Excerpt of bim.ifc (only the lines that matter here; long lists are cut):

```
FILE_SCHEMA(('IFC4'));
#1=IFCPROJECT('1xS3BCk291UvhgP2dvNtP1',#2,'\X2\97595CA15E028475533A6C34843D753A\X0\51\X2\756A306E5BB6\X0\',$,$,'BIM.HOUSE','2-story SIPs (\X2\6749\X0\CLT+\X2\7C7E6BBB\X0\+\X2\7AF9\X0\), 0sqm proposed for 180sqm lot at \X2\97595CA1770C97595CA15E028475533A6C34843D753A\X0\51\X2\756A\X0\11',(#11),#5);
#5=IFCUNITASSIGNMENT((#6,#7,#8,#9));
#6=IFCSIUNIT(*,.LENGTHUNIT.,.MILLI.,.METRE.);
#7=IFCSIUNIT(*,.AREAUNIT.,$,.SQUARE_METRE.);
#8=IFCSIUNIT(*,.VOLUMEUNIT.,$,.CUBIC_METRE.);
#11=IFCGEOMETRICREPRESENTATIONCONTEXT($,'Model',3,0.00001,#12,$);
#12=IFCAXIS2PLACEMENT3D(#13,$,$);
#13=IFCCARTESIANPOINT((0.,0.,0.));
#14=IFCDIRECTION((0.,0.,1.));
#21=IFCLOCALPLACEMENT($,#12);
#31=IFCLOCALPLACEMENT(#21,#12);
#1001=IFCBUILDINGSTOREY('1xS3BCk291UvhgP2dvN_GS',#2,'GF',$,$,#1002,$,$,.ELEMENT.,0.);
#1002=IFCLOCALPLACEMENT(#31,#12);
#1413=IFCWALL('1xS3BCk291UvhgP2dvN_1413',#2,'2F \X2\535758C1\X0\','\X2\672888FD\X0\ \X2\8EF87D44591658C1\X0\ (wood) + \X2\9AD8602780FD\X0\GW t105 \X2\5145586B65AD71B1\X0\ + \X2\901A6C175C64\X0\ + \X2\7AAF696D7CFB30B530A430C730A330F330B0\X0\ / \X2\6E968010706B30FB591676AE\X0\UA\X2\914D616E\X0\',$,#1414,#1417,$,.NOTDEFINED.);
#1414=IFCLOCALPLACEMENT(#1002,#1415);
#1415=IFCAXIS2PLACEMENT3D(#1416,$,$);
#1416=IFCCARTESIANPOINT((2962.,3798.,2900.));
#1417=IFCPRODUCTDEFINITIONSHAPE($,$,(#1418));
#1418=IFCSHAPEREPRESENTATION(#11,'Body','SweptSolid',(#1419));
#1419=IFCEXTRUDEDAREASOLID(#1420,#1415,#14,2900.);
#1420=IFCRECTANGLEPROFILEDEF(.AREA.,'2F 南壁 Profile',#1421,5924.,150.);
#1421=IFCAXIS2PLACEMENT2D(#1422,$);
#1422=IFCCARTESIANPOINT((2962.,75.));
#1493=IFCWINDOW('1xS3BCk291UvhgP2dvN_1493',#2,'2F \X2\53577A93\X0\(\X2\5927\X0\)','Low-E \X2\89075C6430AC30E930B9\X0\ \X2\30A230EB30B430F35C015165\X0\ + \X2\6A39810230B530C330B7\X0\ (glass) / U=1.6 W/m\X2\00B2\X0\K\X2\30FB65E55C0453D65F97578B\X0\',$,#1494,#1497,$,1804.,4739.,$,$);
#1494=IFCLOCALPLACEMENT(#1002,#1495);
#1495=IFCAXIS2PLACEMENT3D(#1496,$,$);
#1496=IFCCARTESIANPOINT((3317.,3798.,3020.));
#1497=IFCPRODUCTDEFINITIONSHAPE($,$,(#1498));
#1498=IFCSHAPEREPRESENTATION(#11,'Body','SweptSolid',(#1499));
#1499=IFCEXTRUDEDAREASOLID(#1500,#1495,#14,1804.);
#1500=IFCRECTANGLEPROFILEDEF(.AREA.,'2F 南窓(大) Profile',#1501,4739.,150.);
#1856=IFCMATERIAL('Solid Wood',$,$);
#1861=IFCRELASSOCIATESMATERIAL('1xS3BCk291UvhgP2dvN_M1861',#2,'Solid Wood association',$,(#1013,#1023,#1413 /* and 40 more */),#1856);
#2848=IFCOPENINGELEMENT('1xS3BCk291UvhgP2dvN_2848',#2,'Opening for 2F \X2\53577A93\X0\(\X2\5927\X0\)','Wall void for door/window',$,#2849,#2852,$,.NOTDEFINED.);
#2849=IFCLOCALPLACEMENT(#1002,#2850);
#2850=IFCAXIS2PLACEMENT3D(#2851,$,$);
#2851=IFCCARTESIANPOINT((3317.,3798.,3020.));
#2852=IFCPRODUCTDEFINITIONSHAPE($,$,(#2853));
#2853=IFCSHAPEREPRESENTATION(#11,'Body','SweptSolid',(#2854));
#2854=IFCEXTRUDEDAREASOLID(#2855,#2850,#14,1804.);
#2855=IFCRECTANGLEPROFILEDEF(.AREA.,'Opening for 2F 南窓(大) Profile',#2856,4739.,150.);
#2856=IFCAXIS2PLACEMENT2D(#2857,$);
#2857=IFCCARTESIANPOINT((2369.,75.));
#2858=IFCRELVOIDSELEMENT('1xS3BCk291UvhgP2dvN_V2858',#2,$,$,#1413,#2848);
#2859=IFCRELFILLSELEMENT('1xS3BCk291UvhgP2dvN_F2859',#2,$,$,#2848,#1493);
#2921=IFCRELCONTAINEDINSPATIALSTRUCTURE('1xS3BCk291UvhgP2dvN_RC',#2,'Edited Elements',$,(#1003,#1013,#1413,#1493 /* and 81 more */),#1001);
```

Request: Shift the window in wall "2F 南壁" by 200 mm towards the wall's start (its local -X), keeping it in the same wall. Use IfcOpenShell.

```python
import ifcopenshell
import ifcopenshell.api.geometry
import ifcopenshell.util.placement

model = ifcopenshell.open("bim.ifc")

window = model.by_id(1493)
opening = window.FillsVoids[0].RelatingOpeningElement
wall = opening.VoidsElements[0].RelatingBuildingElement

wall_matrix = ifcopenshell.util.placement.get_local_placement(wall.ObjectPlacement)
shift = wall_matrix[:3, 0] * -200.0
before = ifcopenshell.util.placement.get_local_placement(window.ObjectPlacement)[:3, 3].copy()

# The window is not placed relative to its opening, so move both.
for product in (opening, window):
    matrix = ifcopenshell.util.placement.get_local_placement(product.ObjectPlacement)
    matrix[:3, 3] += shift
    ifcopenshell.api.geometry.edit_object_placement(model, product=product, matrix=matrix, is_si=False)

after = ifcopenshell.util.placement.get_local_placement(window.ObjectPlacement)[:3, 3]
print("window moved by", (after - before).round(3) + 0.0)

model.write("bim_v2.ifc")
```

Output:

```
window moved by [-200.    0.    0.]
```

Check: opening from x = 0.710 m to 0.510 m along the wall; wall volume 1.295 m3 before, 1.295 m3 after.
